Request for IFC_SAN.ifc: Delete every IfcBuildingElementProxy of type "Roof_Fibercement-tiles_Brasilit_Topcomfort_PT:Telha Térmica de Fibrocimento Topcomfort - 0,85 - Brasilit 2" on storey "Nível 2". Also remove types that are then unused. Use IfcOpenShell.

First a look at what the model holds.

```python
import ifcopenshell
import ifcopenshell.util.element

model = ifcopenshell.open("IFC_SAN.ifc")
print(model.schema)
storey = next(s for s in model.by_type("IfcBuildingStorey") if s.Name == "Nível 2")
proxies = [e for e in ifcopenshell.util.element.get_decomposition(storey) if e.is_a("IfcBuildingElementProxy")]
seen = {}
for e in proxies:
    element_type = ifcopenshell.util.element.get_type(e)
    name = element_type.Name if element_type not in (None, e) else None
    seen[name] = seen.get(name, 0) + 1
for name, count in sorted(seen.items(), key=str):
    print(count, "x", name)
```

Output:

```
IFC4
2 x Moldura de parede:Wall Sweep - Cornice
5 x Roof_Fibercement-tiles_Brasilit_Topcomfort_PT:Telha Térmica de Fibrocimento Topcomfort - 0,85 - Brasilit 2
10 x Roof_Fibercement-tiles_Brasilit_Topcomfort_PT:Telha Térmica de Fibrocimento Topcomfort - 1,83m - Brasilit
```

```python
import ifcopenshell
import ifcopenshell.api.root
import ifcopenshell.util.element

model = ifcopenshell.open("IFC_SAN.ifc")

storey = next(s for s in model.by_type("IfcBuildingStorey") if s.Name == "Nível 2")
proxies = [e for e in ifcopenshell.util.element.get_decomposition(storey) if e.is_a("IfcBuildingElementProxy")]
targets = [e for e in proxies if (t := ifcopenshell.util.element.get_type(e)) not in (None, e) and t.Name == "Roof_Fibercement-tiles_Brasilit_Topcomfort_PT:Telha Térmica de Fibrocimento Topcomfort - 0,85 - Brasilit 2"]
types = {ifcopenshell.util.element.get_type(e) for e in targets} - {None, *targets}

for e in targets:
    ifcopenshell.api.root.remove_product(model, product=e)
print(len(targets), "removed")

unused = [t for t in types if not ifcopenshell.util.element.get_types(t)]
for t in unused:
    ifcopenshell.api.root.remove_product(model, product=t)
print(len(unused), "unused types removed")

model.write("IFC_SAN_v2.ifc")
```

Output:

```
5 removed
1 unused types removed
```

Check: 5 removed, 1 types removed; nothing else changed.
